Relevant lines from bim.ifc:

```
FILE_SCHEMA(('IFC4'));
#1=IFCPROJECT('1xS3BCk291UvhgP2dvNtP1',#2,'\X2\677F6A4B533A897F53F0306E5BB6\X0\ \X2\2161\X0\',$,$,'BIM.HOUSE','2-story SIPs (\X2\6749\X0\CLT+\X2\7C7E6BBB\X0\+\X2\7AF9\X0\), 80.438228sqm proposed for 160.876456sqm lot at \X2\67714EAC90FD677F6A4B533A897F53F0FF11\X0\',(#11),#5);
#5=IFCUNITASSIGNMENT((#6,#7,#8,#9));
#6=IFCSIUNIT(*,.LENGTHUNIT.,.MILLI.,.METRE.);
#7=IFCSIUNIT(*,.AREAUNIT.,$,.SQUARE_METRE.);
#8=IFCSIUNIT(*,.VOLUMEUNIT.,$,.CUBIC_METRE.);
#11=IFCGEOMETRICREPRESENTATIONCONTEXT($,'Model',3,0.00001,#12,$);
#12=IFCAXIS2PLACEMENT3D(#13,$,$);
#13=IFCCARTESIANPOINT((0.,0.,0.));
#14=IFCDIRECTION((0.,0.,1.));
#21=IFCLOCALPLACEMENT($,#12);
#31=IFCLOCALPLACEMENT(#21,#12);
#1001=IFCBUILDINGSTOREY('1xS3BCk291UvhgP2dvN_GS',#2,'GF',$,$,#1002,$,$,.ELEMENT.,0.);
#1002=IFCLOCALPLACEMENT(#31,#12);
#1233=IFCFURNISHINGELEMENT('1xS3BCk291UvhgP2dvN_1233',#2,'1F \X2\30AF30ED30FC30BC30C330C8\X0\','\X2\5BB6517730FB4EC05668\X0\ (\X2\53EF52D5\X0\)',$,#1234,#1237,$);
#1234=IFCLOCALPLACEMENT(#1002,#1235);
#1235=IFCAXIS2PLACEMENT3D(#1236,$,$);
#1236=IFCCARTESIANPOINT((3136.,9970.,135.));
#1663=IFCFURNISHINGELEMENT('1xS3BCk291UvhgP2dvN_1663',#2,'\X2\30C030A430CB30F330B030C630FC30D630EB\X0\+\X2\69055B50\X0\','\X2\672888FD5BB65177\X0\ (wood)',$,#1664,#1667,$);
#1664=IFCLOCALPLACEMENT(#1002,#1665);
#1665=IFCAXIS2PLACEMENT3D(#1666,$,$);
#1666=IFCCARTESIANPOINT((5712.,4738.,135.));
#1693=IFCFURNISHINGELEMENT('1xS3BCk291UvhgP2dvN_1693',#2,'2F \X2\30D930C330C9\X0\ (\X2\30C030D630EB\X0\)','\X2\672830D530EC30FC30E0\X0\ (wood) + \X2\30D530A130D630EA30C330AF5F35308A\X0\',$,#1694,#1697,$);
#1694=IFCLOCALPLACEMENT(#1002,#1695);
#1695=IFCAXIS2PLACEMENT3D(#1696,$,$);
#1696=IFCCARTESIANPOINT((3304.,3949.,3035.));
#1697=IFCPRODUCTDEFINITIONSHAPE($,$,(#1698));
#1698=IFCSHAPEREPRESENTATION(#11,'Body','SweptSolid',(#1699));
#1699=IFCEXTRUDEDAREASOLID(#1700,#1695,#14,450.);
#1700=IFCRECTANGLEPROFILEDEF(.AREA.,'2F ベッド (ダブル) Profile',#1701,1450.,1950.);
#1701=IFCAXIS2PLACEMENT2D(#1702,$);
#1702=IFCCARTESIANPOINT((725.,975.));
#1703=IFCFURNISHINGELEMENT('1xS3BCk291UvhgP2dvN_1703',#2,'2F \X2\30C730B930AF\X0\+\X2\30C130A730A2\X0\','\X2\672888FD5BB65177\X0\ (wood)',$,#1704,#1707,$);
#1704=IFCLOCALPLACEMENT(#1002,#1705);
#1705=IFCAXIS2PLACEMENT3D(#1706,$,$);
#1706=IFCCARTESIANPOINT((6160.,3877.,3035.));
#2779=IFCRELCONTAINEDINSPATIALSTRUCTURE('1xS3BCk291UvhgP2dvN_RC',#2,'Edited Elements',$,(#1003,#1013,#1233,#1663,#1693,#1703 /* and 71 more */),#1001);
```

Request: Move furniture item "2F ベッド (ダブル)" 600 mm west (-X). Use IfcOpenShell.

```python
import ifcopenshell
import ifcopenshell.api.geometry
import ifcopenshell.util.placement

model = ifcopenshell.open("bim.ifc")

item = model.by_guid("1xS3BCk291UvhgP2dvN_1693")
matrix = ifcopenshell.util.placement.get_local_placement(item.ObjectPlacement)
matrix[0, 3] -= 600.0
ifcopenshell.api.geometry.edit_object_placement(model, product=item, matrix=matrix, is_si=False)

print(ifcopenshell.util.placement.get_local_placement(item.ObjectPlacement).round(3) + 0.0)

model.write("bim_v2.ifc")
```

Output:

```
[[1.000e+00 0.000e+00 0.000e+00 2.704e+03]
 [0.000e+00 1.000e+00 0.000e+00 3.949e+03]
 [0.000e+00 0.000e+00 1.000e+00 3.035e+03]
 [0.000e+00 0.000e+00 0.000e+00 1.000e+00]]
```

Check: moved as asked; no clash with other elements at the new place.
